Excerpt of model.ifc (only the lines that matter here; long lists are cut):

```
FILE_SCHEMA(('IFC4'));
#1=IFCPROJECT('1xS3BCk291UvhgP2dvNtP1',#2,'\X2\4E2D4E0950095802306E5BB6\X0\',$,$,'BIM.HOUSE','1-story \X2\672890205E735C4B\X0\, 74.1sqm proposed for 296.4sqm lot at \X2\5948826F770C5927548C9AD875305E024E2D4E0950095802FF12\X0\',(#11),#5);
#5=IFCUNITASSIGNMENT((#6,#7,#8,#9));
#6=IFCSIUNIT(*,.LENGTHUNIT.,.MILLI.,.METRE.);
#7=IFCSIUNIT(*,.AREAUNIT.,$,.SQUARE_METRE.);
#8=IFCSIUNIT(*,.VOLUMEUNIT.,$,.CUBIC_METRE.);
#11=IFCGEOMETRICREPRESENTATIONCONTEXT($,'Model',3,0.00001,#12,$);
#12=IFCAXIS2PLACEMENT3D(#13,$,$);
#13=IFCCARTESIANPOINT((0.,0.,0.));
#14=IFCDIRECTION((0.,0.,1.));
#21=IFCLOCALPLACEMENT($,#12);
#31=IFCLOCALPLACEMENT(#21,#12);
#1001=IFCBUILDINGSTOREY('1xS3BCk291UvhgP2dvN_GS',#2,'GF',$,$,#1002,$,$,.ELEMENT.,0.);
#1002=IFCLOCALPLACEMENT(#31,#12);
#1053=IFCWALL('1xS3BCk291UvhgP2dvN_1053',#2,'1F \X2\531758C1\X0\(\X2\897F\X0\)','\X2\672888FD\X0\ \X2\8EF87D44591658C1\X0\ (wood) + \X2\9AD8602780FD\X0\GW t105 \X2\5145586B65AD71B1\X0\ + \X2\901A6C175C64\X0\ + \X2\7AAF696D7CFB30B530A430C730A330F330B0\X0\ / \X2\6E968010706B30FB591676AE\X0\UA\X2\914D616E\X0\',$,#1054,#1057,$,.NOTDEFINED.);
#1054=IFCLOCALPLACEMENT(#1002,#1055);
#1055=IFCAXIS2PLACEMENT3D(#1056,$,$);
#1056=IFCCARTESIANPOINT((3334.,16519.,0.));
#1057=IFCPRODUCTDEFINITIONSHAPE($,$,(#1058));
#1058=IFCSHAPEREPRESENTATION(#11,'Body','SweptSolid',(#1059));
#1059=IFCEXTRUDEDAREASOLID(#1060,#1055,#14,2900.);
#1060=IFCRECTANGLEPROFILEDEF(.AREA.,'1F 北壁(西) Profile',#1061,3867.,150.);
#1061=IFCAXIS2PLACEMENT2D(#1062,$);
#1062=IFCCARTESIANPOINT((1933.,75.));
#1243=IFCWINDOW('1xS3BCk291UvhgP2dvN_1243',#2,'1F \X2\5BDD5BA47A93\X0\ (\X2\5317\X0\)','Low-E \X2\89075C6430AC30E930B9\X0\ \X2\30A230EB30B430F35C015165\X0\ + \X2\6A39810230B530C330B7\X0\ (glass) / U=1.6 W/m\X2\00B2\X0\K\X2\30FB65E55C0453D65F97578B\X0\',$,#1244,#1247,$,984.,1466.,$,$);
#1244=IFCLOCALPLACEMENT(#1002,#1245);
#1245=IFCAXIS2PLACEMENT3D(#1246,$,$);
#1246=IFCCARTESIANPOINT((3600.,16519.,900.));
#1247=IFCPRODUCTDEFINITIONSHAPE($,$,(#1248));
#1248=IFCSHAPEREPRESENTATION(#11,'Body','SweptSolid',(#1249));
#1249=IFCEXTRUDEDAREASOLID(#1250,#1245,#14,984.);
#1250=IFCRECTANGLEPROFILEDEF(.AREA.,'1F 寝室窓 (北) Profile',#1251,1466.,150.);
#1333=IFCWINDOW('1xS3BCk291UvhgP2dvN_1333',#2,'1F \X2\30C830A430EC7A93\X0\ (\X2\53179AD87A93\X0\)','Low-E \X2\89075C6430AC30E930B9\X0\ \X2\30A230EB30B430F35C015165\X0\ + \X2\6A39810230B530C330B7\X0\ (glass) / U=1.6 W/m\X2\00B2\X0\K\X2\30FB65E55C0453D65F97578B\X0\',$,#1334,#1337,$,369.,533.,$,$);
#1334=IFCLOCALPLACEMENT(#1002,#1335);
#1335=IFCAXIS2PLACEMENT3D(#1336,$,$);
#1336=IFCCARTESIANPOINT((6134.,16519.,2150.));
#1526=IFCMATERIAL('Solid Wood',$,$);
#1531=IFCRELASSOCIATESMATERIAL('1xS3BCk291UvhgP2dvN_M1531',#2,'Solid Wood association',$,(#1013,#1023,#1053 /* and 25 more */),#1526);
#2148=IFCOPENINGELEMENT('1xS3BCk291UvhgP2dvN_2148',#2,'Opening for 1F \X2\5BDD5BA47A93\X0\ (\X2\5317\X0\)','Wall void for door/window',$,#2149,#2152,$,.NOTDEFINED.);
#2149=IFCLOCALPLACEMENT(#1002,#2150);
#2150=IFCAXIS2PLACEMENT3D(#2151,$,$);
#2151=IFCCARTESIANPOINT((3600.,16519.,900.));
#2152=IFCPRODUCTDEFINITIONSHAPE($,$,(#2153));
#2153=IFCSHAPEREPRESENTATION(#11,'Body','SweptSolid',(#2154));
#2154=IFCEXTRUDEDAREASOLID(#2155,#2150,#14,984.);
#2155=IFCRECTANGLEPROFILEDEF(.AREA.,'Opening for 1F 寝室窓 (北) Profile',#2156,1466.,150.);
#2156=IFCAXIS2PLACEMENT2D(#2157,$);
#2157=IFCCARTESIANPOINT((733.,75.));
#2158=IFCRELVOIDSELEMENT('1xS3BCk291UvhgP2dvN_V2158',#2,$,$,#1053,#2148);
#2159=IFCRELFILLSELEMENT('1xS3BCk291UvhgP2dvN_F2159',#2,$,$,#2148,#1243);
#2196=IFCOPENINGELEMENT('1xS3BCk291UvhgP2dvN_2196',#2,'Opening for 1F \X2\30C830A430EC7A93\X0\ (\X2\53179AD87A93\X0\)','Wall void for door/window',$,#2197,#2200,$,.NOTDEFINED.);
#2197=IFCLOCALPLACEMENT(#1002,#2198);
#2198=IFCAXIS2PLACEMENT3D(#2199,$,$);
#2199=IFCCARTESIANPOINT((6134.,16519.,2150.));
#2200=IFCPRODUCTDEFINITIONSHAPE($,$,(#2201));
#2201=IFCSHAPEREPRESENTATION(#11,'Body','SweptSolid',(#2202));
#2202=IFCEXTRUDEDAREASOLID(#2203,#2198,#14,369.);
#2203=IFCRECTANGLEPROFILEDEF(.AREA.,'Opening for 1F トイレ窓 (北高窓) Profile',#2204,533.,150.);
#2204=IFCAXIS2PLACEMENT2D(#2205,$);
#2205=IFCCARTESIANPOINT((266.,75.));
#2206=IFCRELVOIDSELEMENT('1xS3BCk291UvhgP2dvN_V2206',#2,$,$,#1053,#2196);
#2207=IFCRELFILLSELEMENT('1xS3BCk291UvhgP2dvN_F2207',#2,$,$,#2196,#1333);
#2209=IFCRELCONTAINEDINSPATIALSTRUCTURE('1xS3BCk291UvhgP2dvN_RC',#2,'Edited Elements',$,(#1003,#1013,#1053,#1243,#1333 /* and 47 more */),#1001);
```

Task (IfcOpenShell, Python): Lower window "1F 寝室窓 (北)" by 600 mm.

```python
import numpy as np
import ifcopenshell
import ifcopenshell.api.geometry
import ifcopenshell.util.placement
import ifcopenshell.util.unit

model = ifcopenshell.open("model.ifc")
unit_scale = ifcopenshell.util.unit.calculate_unit_scale(model)

window = model.by_guid("1xS3BCk291UvhgP2dvN_1243")
opening = window.FillsVoids[0].RelatingOpeningElement
dz = -0.6 / unit_scale

shift = np.array([0.0, 0.0, dz])
# The window is not placed relative to its opening, so move both.
for product in (opening, window):
    matrix = ifcopenshell.util.placement.get_local_placement(product.ObjectPlacement)
    matrix[:3, 3] += shift
    ifcopenshell.api.geometry.edit_object_placement(model, product=product, matrix=matrix, is_si=False)

print(f"moved by {dz * unit_scale:+.3f} m")

model.write("model-out.ifc")
```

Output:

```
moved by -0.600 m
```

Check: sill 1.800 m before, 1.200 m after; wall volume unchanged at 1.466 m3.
